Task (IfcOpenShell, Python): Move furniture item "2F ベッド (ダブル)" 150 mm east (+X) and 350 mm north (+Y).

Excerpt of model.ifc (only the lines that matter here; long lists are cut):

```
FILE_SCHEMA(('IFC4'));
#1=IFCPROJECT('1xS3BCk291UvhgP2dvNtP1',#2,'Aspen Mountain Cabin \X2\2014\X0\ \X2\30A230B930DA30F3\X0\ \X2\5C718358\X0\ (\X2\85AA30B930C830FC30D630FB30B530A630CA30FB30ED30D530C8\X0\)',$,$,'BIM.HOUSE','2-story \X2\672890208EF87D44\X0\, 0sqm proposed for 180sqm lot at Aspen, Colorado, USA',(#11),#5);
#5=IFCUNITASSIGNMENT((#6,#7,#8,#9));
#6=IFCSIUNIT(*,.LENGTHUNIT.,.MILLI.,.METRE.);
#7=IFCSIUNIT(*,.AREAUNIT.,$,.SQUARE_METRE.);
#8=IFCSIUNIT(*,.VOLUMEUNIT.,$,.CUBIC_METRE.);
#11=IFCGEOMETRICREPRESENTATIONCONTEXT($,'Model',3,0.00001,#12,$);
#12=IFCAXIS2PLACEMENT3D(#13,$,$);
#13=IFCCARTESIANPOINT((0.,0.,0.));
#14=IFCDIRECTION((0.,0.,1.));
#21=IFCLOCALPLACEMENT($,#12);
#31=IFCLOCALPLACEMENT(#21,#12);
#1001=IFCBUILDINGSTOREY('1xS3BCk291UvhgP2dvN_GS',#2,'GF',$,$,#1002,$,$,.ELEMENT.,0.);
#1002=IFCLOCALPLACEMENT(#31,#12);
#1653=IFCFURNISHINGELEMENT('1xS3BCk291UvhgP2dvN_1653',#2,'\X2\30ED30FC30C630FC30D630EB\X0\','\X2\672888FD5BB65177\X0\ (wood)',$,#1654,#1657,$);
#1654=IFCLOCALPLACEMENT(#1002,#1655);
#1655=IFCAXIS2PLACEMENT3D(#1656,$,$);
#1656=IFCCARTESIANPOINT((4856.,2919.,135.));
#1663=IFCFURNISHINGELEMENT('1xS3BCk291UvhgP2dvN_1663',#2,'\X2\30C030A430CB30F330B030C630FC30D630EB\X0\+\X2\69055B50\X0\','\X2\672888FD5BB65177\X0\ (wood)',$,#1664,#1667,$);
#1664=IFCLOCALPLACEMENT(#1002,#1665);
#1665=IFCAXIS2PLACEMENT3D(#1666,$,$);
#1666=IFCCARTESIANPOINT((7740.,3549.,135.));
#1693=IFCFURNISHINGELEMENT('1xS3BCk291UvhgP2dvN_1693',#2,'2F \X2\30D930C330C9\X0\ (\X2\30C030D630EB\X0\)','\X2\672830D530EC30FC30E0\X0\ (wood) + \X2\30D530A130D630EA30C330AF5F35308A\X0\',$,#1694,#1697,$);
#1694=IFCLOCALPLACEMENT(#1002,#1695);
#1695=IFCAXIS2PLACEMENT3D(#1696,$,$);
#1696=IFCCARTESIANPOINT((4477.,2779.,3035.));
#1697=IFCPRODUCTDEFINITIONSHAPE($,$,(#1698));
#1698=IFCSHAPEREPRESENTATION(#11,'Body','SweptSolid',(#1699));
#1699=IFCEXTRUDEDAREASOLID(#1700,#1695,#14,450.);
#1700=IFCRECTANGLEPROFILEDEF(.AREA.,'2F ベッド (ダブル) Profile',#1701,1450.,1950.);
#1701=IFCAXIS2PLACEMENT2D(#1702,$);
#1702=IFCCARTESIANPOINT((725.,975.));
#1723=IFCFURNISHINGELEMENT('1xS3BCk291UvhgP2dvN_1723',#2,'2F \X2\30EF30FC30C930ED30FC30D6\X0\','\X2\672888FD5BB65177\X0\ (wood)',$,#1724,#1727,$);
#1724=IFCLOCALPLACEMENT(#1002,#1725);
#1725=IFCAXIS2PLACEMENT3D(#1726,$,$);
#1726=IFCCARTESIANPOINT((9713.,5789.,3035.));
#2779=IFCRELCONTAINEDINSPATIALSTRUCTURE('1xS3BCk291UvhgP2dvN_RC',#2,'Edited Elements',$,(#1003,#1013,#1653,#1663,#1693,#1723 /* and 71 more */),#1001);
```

```python
import ifcopenshell
import ifcopenshell.api.geometry
import ifcopenshell.util.placement

model = ifcopenshell.open("model.ifc")

item = model.by_guid("1xS3BCk291UvhgP2dvN_1693")
matrix = ifcopenshell.util.placement.get_local_placement(item.ObjectPlacement)
matrix[0, 3] += 150.0
matrix[1, 3] += 350.0
ifcopenshell.api.geometry.edit_object_placement(model, product=item, matrix=matrix, is_si=False)

print(ifcopenshell.util.placement.get_local_placement(item.ObjectPlacement).round(3) + 0.0)

model.write("model_v2.ifc")
```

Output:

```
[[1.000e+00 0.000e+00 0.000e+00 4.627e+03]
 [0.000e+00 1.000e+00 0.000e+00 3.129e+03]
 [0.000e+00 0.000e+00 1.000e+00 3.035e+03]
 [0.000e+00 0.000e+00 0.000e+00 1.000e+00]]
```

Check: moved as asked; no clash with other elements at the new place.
